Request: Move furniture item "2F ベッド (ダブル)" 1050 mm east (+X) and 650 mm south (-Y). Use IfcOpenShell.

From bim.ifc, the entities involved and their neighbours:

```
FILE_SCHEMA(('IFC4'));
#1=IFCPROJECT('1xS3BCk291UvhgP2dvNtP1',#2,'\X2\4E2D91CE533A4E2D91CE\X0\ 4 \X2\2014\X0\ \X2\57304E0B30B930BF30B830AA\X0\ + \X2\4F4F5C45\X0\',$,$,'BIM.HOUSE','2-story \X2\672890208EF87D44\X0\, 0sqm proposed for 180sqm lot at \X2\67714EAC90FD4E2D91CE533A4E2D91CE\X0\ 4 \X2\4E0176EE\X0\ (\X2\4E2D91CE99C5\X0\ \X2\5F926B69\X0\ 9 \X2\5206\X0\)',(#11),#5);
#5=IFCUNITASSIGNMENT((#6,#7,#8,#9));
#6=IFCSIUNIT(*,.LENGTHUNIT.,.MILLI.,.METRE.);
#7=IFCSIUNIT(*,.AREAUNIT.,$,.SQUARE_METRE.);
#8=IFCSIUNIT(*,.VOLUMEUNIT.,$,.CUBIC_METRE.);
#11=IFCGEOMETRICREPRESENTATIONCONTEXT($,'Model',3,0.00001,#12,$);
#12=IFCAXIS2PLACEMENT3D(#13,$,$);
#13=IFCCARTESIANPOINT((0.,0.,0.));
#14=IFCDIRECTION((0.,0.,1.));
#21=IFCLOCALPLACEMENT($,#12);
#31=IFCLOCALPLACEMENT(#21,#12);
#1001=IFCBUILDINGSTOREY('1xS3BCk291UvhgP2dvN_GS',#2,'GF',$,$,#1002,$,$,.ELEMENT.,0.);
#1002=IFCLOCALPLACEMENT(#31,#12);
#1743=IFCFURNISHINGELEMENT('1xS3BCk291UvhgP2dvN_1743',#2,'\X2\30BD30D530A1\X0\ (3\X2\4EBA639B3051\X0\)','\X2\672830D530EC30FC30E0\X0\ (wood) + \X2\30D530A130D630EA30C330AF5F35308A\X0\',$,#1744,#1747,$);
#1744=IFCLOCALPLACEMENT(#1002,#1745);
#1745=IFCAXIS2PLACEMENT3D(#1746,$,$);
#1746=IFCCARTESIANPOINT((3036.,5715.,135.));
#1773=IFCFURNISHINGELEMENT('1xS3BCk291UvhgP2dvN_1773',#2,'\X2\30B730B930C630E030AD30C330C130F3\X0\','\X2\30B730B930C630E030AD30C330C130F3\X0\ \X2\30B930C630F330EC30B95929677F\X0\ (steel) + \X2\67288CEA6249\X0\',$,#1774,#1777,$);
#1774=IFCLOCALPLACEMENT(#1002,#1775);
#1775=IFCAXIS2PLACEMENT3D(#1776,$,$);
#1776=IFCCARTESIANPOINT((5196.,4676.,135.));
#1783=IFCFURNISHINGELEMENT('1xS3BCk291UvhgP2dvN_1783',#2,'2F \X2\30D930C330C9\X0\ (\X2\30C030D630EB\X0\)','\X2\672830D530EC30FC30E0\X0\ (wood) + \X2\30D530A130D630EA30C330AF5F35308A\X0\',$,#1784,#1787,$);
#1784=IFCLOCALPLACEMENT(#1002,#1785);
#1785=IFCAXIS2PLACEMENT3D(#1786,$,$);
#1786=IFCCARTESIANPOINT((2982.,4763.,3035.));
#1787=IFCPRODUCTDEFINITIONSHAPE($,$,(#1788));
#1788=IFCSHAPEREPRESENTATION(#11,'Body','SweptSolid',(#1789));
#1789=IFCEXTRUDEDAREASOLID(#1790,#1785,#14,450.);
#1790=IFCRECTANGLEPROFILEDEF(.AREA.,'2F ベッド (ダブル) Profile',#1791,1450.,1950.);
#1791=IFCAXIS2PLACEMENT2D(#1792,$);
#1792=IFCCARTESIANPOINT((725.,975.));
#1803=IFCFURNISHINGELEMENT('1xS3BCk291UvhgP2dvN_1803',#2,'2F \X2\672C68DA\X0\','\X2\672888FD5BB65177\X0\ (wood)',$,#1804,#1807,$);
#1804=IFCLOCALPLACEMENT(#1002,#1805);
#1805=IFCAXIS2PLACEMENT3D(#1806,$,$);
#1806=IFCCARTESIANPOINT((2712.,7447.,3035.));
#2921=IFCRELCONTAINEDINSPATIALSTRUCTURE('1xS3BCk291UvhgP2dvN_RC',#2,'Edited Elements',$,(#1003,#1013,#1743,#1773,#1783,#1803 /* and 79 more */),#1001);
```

```python
import ifcopenshell
import ifcopenshell.api.geometry
import ifcopenshell.util.placement
import ifcopenshell.util.unit

model = ifcopenshell.open("bim.ifc")
unit_scale = ifcopenshell.util.unit.calculate_unit_scale(model)

item = model.by_id(1783)
matrix = ifcopenshell.util.placement.get_local_placement(item.ObjectPlacement)
matrix[0, 3] += 1.05 / unit_scale
matrix[1, 3] -= 0.65 / unit_scale
ifcopenshell.api.geometry.edit_object_placement(model, product=item, matrix=matrix, is_si=False)

print(ifcopenshell.util.placement.get_local_placement(item.ObjectPlacement).round(3) + 0.0)

model.write("bim_updated.ifc")
```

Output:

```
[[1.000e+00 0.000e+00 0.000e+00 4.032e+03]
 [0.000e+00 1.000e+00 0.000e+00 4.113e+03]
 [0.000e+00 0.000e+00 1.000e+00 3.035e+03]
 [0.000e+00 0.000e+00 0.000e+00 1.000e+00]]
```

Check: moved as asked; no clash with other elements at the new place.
